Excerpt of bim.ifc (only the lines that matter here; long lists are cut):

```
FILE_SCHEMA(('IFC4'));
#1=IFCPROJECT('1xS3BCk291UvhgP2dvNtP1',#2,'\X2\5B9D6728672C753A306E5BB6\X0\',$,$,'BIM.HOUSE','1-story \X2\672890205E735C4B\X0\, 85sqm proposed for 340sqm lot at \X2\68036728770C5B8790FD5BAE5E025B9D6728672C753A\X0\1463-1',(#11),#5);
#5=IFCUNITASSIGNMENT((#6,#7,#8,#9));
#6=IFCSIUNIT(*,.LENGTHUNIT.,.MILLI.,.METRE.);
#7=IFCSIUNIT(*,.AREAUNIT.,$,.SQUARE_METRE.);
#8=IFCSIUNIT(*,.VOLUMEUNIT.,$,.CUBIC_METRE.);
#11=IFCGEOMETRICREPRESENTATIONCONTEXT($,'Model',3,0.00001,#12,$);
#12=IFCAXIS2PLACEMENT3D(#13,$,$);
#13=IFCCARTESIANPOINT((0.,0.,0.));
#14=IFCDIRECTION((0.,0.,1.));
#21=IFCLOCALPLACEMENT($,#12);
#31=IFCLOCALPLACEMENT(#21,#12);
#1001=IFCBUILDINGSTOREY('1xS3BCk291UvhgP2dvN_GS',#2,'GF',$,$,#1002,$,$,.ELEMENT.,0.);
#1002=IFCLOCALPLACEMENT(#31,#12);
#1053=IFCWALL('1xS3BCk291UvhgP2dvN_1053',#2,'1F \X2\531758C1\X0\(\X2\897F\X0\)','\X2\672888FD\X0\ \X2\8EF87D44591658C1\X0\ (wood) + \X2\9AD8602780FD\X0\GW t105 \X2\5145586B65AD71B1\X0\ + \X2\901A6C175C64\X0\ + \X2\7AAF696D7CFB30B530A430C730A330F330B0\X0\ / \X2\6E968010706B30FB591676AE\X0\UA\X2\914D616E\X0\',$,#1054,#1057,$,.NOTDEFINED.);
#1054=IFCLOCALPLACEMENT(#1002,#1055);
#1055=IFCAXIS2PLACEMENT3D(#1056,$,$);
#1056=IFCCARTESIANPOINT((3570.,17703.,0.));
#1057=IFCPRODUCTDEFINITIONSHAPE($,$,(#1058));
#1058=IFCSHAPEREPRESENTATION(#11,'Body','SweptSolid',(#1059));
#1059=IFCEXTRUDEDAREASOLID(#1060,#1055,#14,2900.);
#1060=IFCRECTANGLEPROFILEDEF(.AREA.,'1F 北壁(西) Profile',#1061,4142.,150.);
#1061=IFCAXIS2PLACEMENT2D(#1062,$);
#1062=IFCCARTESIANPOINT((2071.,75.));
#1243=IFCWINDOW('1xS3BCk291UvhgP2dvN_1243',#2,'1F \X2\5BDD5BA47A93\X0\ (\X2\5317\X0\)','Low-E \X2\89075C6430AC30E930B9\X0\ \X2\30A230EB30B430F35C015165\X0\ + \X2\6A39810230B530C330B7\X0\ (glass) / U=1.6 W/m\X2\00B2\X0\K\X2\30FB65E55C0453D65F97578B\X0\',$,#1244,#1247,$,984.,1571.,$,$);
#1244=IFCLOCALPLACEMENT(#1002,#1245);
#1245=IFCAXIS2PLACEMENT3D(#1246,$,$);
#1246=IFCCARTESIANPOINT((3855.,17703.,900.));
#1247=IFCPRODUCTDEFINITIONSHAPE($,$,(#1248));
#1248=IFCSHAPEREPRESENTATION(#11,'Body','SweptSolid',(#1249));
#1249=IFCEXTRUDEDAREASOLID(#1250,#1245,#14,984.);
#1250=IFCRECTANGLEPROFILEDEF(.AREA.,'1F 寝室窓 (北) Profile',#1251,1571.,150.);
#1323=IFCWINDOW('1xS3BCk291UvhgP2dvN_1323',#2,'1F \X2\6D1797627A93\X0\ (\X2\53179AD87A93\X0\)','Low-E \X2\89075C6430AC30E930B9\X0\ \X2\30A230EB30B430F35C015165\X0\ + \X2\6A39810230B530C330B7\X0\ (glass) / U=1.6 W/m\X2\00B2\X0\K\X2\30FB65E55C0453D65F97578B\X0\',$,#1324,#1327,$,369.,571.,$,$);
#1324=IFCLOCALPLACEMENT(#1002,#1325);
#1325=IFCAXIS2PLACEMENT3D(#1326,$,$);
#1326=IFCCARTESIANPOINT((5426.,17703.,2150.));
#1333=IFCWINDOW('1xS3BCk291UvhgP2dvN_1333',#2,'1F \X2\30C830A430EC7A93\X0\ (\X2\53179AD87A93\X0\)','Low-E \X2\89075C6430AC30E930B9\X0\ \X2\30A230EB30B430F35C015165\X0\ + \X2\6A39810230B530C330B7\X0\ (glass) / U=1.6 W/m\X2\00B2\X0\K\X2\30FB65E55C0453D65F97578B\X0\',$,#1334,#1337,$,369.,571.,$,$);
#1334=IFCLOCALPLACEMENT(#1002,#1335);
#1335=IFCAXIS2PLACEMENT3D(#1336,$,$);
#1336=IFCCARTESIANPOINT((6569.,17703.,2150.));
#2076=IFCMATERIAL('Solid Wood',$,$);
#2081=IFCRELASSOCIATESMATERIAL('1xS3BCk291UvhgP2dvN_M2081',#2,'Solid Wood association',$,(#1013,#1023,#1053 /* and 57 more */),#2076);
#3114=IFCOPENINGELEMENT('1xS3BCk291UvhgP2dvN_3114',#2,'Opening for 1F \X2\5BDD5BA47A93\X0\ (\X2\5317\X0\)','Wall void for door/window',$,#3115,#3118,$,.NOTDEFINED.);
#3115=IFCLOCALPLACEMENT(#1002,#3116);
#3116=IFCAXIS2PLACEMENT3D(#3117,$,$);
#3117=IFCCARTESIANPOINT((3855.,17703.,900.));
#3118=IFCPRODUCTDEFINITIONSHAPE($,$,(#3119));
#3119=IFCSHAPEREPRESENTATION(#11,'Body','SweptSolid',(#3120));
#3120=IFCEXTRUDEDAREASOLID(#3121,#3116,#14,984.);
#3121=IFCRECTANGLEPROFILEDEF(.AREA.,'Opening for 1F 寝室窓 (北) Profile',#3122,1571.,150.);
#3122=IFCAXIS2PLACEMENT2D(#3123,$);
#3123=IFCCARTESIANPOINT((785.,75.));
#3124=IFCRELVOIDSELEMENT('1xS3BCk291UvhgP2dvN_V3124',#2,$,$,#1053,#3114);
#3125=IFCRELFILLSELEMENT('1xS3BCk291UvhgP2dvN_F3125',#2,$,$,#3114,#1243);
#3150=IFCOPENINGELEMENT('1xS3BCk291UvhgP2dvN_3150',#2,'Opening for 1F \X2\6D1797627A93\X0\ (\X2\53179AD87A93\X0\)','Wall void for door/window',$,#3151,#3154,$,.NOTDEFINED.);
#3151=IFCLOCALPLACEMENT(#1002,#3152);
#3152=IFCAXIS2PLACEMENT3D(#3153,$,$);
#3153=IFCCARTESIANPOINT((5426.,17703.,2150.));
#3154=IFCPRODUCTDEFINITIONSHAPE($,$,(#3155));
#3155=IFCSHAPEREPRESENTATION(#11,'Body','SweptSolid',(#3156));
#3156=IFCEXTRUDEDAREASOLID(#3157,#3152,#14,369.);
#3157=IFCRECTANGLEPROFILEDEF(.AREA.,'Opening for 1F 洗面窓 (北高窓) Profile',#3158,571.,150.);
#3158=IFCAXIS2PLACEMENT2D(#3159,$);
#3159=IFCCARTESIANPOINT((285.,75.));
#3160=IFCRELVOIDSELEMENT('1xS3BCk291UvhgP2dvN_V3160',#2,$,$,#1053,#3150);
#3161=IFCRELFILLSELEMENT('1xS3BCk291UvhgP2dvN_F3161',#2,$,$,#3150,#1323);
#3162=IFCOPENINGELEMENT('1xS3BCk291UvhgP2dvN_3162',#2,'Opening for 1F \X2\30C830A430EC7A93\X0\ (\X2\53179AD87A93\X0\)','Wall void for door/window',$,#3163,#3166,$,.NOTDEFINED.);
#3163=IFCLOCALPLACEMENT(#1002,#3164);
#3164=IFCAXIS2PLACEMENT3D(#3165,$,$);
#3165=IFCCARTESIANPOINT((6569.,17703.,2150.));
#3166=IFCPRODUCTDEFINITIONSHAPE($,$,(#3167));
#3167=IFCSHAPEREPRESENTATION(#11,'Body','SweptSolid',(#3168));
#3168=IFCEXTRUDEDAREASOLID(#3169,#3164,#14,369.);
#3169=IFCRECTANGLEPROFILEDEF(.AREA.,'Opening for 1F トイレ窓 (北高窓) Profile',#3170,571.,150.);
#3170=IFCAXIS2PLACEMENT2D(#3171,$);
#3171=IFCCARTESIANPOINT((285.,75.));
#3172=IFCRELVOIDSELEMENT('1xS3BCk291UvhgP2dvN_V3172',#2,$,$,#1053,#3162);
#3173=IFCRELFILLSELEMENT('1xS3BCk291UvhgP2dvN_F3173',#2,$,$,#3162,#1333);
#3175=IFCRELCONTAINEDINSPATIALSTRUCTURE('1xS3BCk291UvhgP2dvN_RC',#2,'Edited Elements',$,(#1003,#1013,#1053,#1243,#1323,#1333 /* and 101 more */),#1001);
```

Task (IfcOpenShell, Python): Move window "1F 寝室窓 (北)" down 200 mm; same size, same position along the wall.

```python
import numpy as np
import ifcopenshell
import ifcopenshell.api.geometry
import ifcopenshell.util.placement
import ifcopenshell.util.unit

model = ifcopenshell.open("bim.ifc")
unit_scale = ifcopenshell.util.unit.calculate_unit_scale(model)

window = model.by_guid("1xS3BCk291UvhgP2dvN_1243")
opening = window.FillsVoids[0].RelatingOpeningElement
dz = -200.0

shift = np.array([0.0, 0.0, dz])
# The window is not placed relative to its opening, so move both.
for product in (opening, window):
    matrix = ifcopenshell.util.placement.get_local_placement(product.ObjectPlacement)
    matrix[:3, 3] += shift
    ifcopenshell.api.geometry.edit_object_placement(model, product=product, matrix=matrix, is_si=False)

print(f"moved by {dz * unit_scale:+.3f} m")

model.write("bim-out.ifc")
```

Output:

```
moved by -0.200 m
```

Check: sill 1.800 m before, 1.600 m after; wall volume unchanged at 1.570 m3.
